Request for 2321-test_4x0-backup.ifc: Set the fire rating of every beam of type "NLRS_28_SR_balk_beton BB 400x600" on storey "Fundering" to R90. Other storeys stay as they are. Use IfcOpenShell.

First a look at what the model holds.

```python
import ifcopenshell
import ifcopenshell.util.element

model = ifcopenshell.open("2321-test_4x0-backup.ifc")
print(model.schema)
storey = next(s for s in model.by_type("IfcBuildingStorey") if s.Name == "Fundering")
beams = [e for e in ifcopenshell.util.element.get_decomposition(storey) if e.is_a("IfcBeam")]
seen = {}
for e in beams:
    element_type = ifcopenshell.util.element.get_type(e)
    key = (element_type.Name if element_type != e and element_type else None, ifcopenshell.util.element.get_pset(e, "Pset_BeamCommon", "FireRating"))
    seen[key] = seen.get(key, 0) + 1
for (name, value), count in sorted(seen.items(), key=str):
    print(count, "x", name, "|", value)
```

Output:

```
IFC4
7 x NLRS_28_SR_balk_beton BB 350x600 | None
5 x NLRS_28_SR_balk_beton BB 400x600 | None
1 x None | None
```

```python
import ifcopenshell
import ifcopenshell.api.pset
import ifcopenshell.util.element

model = ifcopenshell.open("2321-test_4x0-backup.ifc")

storey = next(s for s in model.by_type("IfcBuildingStorey") if s.Name == "Fundering")
beams = [e for e in ifcopenshell.util.element.get_decomposition(storey) if e.is_a("IfcBeam")]

count = 0
for e in beams:
    element_type = ifcopenshell.util.element.get_type(e)
    if element_type in (None, e) or element_type.Name != "NLRS_28_SR_balk_beton BB 400x600":
        continue
    # add_pset returns the element's existing set when there is one.
    pset = ifcopenshell.api.pset.add_pset(model, product=e, name="Pset_BeamCommon")
    ifcopenshell.api.pset.edit_pset(model, pset=pset, properties={"FireRating": "R90"})
    count += 1

print(count, "beams updated")

model.write("2321-test_4x0-backup-out.ifc")
```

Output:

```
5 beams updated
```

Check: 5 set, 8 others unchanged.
